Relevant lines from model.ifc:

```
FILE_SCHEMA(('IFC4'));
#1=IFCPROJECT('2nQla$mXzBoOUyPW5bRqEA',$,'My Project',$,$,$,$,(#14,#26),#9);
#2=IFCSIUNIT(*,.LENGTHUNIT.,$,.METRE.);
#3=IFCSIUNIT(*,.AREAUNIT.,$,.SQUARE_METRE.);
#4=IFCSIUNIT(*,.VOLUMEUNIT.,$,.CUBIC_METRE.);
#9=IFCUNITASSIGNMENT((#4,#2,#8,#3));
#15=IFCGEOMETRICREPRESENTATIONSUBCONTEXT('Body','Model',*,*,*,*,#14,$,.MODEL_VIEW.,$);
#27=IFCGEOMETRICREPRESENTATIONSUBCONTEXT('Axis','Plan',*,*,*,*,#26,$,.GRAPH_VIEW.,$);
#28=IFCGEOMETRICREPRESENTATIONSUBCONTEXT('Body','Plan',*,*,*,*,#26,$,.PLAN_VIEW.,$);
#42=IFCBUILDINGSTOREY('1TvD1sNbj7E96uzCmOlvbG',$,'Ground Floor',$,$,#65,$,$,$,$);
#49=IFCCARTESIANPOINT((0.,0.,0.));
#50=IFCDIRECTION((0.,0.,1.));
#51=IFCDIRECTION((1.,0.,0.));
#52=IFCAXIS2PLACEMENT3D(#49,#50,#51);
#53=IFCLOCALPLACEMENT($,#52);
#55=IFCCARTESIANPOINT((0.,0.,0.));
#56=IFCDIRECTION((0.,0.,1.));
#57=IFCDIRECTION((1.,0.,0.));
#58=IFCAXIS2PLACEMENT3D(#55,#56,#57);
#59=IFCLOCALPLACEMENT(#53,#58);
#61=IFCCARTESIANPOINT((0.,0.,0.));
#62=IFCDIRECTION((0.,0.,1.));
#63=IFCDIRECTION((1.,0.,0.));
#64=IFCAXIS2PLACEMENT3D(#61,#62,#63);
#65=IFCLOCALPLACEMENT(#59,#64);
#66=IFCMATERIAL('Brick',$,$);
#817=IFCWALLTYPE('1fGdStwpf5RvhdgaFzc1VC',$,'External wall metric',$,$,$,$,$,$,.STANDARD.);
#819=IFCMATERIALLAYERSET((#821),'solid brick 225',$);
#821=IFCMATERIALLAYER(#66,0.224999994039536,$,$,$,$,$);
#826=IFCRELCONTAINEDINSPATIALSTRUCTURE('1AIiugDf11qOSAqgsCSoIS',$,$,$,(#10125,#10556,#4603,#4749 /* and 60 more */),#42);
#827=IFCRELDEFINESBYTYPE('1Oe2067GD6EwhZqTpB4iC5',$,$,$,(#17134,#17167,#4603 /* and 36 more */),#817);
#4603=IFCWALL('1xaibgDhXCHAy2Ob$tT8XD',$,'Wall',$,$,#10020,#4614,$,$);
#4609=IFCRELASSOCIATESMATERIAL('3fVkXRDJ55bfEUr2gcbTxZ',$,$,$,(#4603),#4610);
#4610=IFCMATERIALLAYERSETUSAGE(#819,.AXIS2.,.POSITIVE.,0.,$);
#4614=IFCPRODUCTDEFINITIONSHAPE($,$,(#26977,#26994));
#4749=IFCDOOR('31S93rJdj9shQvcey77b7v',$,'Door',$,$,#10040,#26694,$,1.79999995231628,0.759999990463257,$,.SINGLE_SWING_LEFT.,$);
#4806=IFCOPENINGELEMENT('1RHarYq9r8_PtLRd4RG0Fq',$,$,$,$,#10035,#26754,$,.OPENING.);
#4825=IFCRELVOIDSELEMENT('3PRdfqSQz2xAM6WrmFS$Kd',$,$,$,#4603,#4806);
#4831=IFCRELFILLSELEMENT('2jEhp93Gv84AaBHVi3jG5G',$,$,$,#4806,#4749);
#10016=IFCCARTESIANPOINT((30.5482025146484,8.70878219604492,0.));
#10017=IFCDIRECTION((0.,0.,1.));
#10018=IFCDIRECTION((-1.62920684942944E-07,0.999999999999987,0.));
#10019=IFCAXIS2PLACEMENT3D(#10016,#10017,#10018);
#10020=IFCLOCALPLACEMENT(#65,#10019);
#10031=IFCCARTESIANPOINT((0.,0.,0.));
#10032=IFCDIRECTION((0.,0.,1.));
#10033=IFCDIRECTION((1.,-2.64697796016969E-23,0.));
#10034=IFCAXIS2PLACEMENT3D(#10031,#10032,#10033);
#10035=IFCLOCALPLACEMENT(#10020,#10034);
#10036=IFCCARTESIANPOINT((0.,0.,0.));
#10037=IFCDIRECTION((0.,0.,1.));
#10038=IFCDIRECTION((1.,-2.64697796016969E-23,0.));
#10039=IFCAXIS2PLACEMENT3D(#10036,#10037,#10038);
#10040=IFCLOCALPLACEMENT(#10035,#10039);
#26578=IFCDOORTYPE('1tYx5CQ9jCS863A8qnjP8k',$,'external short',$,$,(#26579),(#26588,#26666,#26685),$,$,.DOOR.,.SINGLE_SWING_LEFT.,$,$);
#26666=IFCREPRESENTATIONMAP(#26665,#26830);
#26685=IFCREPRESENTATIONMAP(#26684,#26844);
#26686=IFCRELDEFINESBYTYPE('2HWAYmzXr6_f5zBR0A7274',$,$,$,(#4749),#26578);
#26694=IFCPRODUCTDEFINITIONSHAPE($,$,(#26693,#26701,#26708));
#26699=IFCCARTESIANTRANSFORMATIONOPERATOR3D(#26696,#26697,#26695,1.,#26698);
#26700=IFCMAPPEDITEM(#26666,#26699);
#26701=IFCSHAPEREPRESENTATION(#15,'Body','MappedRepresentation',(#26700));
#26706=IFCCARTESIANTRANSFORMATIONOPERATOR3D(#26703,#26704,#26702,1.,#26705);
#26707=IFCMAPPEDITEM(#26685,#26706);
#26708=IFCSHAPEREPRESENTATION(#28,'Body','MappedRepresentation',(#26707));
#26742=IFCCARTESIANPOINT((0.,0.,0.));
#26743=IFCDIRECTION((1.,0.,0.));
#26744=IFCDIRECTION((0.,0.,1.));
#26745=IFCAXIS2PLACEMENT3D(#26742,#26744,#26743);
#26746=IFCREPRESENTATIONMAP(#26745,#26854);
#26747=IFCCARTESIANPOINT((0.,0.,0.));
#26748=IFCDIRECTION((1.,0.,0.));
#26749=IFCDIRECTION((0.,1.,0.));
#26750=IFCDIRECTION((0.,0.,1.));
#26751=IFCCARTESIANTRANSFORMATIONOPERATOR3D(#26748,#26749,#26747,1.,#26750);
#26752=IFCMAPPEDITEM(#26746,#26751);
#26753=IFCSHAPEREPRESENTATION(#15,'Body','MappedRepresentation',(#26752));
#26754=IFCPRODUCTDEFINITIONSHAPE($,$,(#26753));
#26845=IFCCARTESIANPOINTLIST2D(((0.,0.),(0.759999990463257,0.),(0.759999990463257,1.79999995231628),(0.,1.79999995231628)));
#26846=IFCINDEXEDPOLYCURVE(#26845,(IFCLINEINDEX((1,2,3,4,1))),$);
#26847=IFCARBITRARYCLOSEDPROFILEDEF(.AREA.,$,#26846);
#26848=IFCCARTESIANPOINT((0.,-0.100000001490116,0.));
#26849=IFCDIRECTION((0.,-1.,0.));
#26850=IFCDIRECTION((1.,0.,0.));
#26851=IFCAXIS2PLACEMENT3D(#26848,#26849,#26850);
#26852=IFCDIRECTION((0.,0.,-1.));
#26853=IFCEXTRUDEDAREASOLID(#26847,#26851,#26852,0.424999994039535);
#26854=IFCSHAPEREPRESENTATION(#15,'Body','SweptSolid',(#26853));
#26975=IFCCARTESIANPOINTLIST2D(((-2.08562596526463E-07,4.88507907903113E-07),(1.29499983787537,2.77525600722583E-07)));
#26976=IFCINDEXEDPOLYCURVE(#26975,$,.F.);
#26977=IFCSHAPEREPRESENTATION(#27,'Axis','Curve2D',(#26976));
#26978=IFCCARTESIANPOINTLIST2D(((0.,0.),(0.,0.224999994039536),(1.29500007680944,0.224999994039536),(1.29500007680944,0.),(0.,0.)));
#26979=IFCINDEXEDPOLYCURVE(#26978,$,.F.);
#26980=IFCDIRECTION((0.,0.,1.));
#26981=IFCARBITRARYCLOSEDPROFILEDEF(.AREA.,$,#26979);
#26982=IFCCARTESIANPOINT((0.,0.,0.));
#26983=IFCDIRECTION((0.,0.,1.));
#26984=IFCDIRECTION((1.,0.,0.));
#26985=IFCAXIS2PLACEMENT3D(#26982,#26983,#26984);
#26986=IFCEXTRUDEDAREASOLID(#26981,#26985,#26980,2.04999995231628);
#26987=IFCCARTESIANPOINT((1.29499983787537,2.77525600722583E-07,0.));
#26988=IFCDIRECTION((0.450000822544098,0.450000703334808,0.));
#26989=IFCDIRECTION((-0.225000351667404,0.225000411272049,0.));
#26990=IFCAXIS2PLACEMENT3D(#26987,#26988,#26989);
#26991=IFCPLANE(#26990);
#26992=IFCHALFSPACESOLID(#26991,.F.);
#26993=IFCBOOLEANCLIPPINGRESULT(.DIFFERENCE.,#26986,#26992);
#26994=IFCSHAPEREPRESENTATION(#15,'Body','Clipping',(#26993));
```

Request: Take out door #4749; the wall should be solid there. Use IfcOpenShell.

```python
import ifcopenshell
import ifcopenshell.api.feature
import ifcopenshell.api.root
import ifcopenshell.geom
import ifcopenshell.util.shape

model = ifcopenshell.open("model.ifc")
settings = ifcopenshell.geom.settings()


def volume(element):
    """Net volume in cubic metres, openings subtracted."""
    shape = ifcopenshell.geom.create_shape(settings, element)
    return ifcopenshell.util.shape.get_volume(shape.geometry)


door = model.by_guid("31S93rJdj9shQvcey77b7v")
opening = door.FillsVoids[0].RelatingOpeningElement
wall = opening.VoidsElements[0].RelatingBuildingElement
before = volume(wall)

ifcopenshell.api.root.remove_product(model, product=door)
ifcopenshell.api.feature.remove_feature(model, feature=opening)

after = volume(wall)

print(f"wall volume {before:.3f} -> {after:.3f} m3")

model.write("model_rev.ifc")
```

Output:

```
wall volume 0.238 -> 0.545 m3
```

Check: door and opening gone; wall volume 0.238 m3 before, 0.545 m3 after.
